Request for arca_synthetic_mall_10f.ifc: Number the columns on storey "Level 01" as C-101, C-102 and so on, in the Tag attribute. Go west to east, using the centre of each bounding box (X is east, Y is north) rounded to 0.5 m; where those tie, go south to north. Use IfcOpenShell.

First a look at what the model holds.

```python
import ifcopenshell
import ifcopenshell.util.element
import ifcopenshell.util.placement

model = ifcopenshell.open("arca_synthetic_mall_10f.ifc")
print(model.schema)
storey = next(s for s in model.by_type("IfcBuildingStorey") if s.Name == "Level 01")
columns = [e for e in ifcopenshell.util.element.get_decomposition(storey) if e.is_a("IfcColumn")]
for e in sorted(columns, key=lambda e: e.id()):
    origin = ifcopenshell.util.placement.get_local_placement(e.ObjectPlacement)[:3, 3]
    print(e.id(), e.Tag, e.Name, origin.round(2) + 0.0, sep=" | ")
```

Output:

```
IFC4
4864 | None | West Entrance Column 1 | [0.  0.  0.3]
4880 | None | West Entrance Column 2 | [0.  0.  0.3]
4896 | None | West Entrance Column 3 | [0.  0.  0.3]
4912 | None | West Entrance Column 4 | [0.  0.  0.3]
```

```python
import ifcopenshell
import ifcopenshell.geom
import ifcopenshell.util.element
import ifcopenshell.util.shape

model = ifcopenshell.open("arca_synthetic_mall_10f.ifc")
settings = ifcopenshell.geom.settings()
settings.set("use-world-coords", True)


def centre(element):
    shape = ifcopenshell.geom.create_shape(settings, element)
    return ifcopenshell.util.shape.get_bbox_centroid(shape.geometry)


storey = next(s for s in model.by_type("IfcBuildingStorey") if s.Name == "Level 01")
columns = [e for e in ifcopenshell.util.element.get_decomposition(storey) if e.is_a("IfcColumn")]

# Insertion points can sit at a corner or the storey origin, so sort by the geometry (in metres).
centres = {e: centre(e) for e in columns}
columns.sort(key=lambda e: (round(centres[e][0] / 0.5), centres[e][1]))

for i, e in enumerate(columns, start=1):
    number = f"C-1{i:02d}"
    e.Tag = number
    print(e.id(), number)

model.write("arca_synthetic_mall_10f_v2.ifc")
```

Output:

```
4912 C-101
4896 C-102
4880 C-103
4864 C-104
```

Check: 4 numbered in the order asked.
